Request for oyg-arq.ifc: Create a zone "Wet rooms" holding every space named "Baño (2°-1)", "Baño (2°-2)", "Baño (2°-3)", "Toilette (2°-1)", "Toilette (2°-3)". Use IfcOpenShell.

First a look at what the model holds.

```python
import ifcopenshell

model = ifcopenshell.open("oyg-arq.ifc")
print(model.schema)
seen = {}
for space in model.by_type("IfcSpace"):
    seen[space.LongName] = seen.get(space.LongName, 0) + 1
for name, count in sorted(seen.items(), key=str):
    print(count, "x", name)
print("zones:", [z.Name for z in model.by_type("IfcZone")][:20])
```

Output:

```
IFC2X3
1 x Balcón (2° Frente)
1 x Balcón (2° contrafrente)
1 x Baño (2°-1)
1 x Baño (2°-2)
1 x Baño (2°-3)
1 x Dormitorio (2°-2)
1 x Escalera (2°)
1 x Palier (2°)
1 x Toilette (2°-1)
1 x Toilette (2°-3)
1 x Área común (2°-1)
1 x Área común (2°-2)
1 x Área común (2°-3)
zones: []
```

```python
import ifcopenshell
import ifcopenshell.api.group
import ifcopenshell.api.root

model = ifcopenshell.open("oyg-arq.ifc")

names = {"Baño (2°-1)", "Baño (2°-2)", "Baño (2°-3)", "Toilette (2°-1)", "Toilette (2°-3)"}
spaces = [s for s in model.by_type("IfcSpace") if s.LongName in names]

zone = ifcopenshell.api.root.create_entity(model, ifc_class="IfcZone", name="Wet rooms")
ifcopenshell.api.group.assign_group(model, products=spaces, group=zone)
print(len(spaces), "spaces in", zone.Name)

model.write("oyg-arq_rev.ifc")
```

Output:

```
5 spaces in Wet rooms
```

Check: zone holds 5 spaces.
